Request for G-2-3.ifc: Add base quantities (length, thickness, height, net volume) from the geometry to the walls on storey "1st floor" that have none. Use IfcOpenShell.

First a look at what the model holds.

```python
import ifcopenshell
import ifcopenshell.util.element
import ifcopenshell.util.unit

model = ifcopenshell.open("G-2-3.ifc")
print(model.schema)
for unit_type in ("LENGTHUNIT", "AREAUNIT", "VOLUMEUNIT"):
    print(unit_type, ifcopenshell.util.unit.calculate_unit_scale(model, unit_type))
storey = next(s for s in model.by_type("IfcBuildingStorey") if s.Name == "1st floor")
walls = [e for e in ifcopenshell.util.element.get_decomposition(storey) if e.is_a("IfcWall")]
for e in sorted(walls, key=lambda e: e.id()):
    print(e.id(), e.is_a(), e.Name, list(ifcopenshell.util.element.get_psets(e, qtos_only=True)), sep=" | ")
```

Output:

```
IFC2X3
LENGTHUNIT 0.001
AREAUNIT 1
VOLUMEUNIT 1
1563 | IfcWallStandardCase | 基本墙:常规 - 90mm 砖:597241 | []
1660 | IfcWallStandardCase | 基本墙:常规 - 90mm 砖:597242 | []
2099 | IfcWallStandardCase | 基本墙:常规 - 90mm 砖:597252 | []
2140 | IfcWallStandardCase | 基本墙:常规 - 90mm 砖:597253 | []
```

```python
import ifcopenshell
import ifcopenshell.api.pset
import ifcopenshell.geom
import ifcopenshell.util.element
import ifcopenshell.util.shape
import ifcopenshell.util.unit

model = ifcopenshell.open("G-2-3.ifc")
unit_scale = ifcopenshell.util.unit.calculate_unit_scale(model)
volume_scale = ifcopenshell.util.unit.calculate_unit_scale(model, "VOLUMEUNIT")
settings = ifcopenshell.geom.settings()

storey = next(s for s in model.by_type("IfcBuildingStorey") if s.Name == "1st floor")
walls = [e for e in ifcopenshell.util.element.get_decomposition(storey) if e.is_a("IfcWall")]

for e in sorted(walls, key=lambda e: e.id()):
    if ifcopenshell.util.element.get_psets(e, qtos_only=True, should_inherit=False):
        continue
    # Geometry comes back in metres, in the element's own axes.
    shape = ifcopenshell.geom.create_shape(settings, e)
    values = {
        "Length": ifcopenshell.util.shape.get_x(shape.geometry) / unit_scale,
        "Width": ifcopenshell.util.shape.get_y(shape.geometry) / unit_scale,
        "Height": ifcopenshell.util.shape.get_z(shape.geometry) / unit_scale,
        "NetVolume": ifcopenshell.util.shape.get_volume(shape.geometry) / volume_scale,
    }
    qto = ifcopenshell.api.pset.add_qto(model, product=e, name="BaseQuantities")
    ifcopenshell.api.pset.edit_qto(model, qto=qto, properties=values)
    print(e.id(), {k: round(v, 3) for k, v in values.items()})

model.write("G-2-3_updated.ifc")
```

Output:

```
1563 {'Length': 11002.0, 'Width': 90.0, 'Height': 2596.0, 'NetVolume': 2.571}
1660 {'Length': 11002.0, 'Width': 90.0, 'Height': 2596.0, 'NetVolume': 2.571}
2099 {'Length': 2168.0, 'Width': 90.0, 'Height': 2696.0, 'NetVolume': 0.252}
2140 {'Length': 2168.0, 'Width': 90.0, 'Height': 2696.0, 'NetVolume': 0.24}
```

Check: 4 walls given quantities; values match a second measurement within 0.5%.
